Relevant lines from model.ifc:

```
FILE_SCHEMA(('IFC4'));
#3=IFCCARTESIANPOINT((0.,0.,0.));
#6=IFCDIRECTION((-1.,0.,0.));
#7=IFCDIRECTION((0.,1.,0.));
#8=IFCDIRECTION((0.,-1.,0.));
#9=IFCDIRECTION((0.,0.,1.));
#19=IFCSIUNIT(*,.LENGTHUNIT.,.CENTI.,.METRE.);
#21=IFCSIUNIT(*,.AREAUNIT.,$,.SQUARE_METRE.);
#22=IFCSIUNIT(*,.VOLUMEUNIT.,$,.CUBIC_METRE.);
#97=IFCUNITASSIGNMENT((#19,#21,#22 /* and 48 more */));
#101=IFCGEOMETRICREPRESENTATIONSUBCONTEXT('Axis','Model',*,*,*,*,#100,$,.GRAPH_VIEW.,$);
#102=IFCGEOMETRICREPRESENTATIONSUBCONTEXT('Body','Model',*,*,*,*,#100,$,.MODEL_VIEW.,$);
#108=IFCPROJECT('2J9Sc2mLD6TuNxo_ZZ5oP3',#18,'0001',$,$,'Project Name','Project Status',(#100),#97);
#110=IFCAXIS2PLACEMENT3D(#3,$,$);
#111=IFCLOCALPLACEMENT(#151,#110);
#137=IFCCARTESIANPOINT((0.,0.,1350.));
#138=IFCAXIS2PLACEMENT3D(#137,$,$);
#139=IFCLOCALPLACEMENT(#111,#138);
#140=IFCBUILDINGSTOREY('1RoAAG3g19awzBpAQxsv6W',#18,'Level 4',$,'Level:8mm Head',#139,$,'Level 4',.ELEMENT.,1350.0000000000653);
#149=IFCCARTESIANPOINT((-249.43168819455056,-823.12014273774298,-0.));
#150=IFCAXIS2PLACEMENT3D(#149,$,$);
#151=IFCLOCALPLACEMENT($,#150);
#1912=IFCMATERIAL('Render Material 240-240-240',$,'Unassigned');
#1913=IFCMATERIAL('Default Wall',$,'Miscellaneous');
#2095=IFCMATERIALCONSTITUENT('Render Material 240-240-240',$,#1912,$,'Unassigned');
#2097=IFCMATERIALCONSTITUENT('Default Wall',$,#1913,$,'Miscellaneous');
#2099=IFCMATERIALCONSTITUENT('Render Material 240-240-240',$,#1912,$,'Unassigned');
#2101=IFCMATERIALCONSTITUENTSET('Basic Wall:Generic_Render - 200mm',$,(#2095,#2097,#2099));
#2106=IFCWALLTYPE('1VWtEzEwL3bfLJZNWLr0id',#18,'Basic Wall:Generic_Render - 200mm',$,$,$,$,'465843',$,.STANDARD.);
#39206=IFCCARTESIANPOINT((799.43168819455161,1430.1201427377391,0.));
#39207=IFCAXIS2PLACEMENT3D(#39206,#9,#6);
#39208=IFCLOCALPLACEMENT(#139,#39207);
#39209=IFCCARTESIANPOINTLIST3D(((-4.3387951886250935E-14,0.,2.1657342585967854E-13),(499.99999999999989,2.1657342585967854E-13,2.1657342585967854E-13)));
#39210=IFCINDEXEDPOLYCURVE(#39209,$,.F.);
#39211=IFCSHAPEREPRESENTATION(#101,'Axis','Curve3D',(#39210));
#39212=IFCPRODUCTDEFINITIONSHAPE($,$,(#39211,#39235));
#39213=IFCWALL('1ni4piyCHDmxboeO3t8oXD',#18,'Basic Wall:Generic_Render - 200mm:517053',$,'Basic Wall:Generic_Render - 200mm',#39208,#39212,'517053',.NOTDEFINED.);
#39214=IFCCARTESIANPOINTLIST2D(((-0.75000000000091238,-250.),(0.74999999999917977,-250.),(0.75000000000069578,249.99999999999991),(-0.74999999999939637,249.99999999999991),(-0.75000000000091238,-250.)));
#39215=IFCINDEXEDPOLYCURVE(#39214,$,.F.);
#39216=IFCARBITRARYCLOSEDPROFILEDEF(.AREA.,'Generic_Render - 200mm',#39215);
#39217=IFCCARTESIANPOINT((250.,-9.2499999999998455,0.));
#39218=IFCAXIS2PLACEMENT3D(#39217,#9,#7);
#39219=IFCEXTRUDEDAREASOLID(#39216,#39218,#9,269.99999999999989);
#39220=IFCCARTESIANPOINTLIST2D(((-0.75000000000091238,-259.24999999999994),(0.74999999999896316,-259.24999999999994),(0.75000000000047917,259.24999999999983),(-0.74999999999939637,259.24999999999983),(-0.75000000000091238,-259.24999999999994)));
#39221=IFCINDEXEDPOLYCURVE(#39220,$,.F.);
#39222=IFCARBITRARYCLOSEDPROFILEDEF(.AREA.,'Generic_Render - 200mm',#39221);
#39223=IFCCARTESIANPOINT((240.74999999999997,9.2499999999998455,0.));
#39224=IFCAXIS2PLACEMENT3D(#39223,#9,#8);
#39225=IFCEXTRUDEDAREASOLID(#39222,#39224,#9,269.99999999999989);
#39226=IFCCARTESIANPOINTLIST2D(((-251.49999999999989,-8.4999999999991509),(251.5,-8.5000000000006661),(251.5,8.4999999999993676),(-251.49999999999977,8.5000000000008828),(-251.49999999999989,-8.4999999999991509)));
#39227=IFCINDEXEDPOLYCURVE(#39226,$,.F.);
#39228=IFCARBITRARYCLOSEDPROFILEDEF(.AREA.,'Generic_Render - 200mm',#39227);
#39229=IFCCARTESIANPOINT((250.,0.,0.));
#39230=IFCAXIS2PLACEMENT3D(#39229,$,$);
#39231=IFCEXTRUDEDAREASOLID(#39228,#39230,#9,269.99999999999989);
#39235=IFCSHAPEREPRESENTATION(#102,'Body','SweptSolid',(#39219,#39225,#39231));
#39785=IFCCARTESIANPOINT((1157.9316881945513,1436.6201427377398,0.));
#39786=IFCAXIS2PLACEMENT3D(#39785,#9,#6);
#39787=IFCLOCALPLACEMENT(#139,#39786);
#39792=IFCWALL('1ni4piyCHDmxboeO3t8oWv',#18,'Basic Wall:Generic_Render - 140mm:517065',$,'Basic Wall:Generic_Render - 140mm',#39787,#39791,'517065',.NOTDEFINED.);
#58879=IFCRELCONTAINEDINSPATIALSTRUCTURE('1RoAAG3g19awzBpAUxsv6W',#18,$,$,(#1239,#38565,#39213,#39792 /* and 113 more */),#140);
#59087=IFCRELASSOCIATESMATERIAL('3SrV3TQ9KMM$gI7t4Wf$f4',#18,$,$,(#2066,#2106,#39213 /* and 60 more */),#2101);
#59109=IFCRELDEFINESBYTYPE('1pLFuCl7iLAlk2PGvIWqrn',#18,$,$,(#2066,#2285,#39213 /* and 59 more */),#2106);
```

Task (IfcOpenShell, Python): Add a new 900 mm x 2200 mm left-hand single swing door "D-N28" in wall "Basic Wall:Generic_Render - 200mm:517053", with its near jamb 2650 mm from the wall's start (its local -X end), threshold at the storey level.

```python
import numpy as np
import ifcopenshell
import ifcopenshell.api.feature
import ifcopenshell.api.geometry
import ifcopenshell.api.root
import ifcopenshell.api.spatial
import ifcopenshell.geom
import ifcopenshell.util.element
import ifcopenshell.util.placement
import ifcopenshell.util.representation
import ifcopenshell.util.shape
import ifcopenshell.util.unit

model = ifcopenshell.open("model.ifc")
unit_scale = ifcopenshell.util.unit.calculate_unit_scale(model)
settings = ifcopenshell.geom.settings()


def volume(element):
    """Net volume in cubic metres, openings subtracted."""
    shape = ifcopenshell.geom.create_shape(settings, element)
    return ifcopenshell.util.shape.get_volume(shape.geometry)


wall = model.by_guid("1ni4piyCHDmxboeO3t8oXD")
storey = ifcopenshell.util.element.get_container(wall, ifc_class="IfcBuildingStorey")
context = ifcopenshell.util.representation.get_context(model, "Model", "Body", "MODEL_VIEW")
before = volume(wall)

width, height, from_end, sill = 0.9, 2.2, 2.65, 0.0  # metres

# The wall runs along its own X axis, and the end named is its -X end.
wall_shape = ifcopenshell.geom.create_shape(settings, wall)
x, y, z = ifcopenshell.util.shape.get_vertices(wall_shape.geometry).T
start = x.min() + from_end
face, thickness = float(y.min()), float(y.max() - y.min())
wall_matrix = ifcopenshell.util.placement.get_local_placement(wall.ObjectPlacement)
level = ifcopenshell.util.placement.get_local_placement(storey.ObjectPlacement)[2, 3]


def in_wall(x, y):
    """Placement at x, y metres in the wall's axes, at sill height."""
    matrix = wall_matrix.copy()
    matrix[:, 3] = wall_matrix @ np.array([x / unit_scale, y / unit_scale, 0.0, 1.0])
    matrix[2, 3] = level + sill / unit_scale
    return matrix


# Opening: a box that overshoots both wall faces by 50 mm.
opening = ifcopenshell.api.root.create_entity(model, ifc_class="IfcOpeningElement", predefined_type="OPENING")
box = ifcopenshell.api.geometry.add_wall_representation(
    model, context=context, length=width, height=height, thickness=thickness + 0.1
)
ifcopenshell.api.geometry.assign_representation(model, product=opening, representation=box)
ifcopenshell.api.geometry.edit_object_placement(model, product=opening, matrix=in_wall(start, face - 0.05), is_si=False)
ifcopenshell.api.feature.add_feature(model, feature=opening, element=wall)

door = ifcopenshell.api.root.create_entity(model, ifc_class="IfcDoor", name="D-N28", predefined_type="DOOR")
door.OverallWidth, door.OverallHeight = width / unit_scale, height / unit_scale
door.OperationType = "SINGLE_SWING_LEFT"
body = ifcopenshell.api.geometry.add_door_representation(
    model,
    context=context,
    overall_width=door.OverallWidth,
    overall_height=door.OverallHeight,
    operation_type="SINGLE_SWING_LEFT",
    lining_properties={"LiningDepth": thickness / unit_scale, "ThresholdDepth": thickness / unit_scale},
)
ifcopenshell.api.geometry.assign_representation(model, product=door, representation=body)
ifcopenshell.api.spatial.assign_container(model, products=[door], relating_structure=storey)
ifcopenshell.api.feature.add_filling(model, opening=opening, element=door)

# The lining spans the wall, so the door starts at the wall face.
ifcopenshell.api.geometry.edit_object_placement(model, product=door, matrix=in_wall(start, face), is_si=False)

after = volume(wall)

print(f"wall volume {before:.3f} -> {after:.3f} m3")

model.write("model_rev.ifc")
```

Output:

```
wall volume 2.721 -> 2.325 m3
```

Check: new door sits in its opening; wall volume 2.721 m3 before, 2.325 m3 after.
